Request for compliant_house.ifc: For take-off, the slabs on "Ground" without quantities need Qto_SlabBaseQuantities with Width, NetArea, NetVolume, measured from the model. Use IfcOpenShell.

First a look at what the model holds.

```python
import ifcopenshell
import ifcopenshell.util.element
import ifcopenshell.util.unit

model = ifcopenshell.open("compliant_house.ifc")
print(model.schema)
for unit_type in ("LENGTHUNIT", "AREAUNIT", "VOLUMEUNIT"):
    print(unit_type, ifcopenshell.util.unit.calculate_unit_scale(model, unit_type))
storey = next(s for s in model.by_type("IfcBuildingStorey") if s.Name == "Ground")
slabs = [e for e in ifcopenshell.util.element.get_decomposition(storey) if e.is_a("IfcSlab")]
for e in sorted(slabs, key=lambda e: e.id()):
    print(e.id(), e.is_a(), e.Name, list(ifcopenshell.util.element.get_psets(e, qtos_only=True)), sep=" | ")
```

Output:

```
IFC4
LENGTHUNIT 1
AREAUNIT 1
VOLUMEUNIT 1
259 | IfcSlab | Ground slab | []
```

```python
import ifcopenshell
import ifcopenshell.api.pset
import ifcopenshell.geom
import ifcopenshell.util.element
import ifcopenshell.util.shape
import ifcopenshell.util.unit

model = ifcopenshell.open("compliant_house.ifc")
unit_scale = ifcopenshell.util.unit.calculate_unit_scale(model)
area_scale = ifcopenshell.util.unit.calculate_unit_scale(model, "AREAUNIT")
volume_scale = ifcopenshell.util.unit.calculate_unit_scale(model, "VOLUMEUNIT")
settings = ifcopenshell.geom.settings()

storey = next(s for s in model.by_type("IfcBuildingStorey") if s.Name == "Ground")
slabs = [e for e in ifcopenshell.util.element.get_decomposition(storey) if e.is_a("IfcSlab")]

for e in sorted(slabs, key=lambda e: e.id()):
    if ifcopenshell.util.element.get_psets(e, qtos_only=True, should_inherit=False):
        continue
    # Geometry comes back in metres, in the element's own axes.
    shape = ifcopenshell.geom.create_shape(settings, e)
    values = {
        "Width": ifcopenshell.util.shape.get_z(shape.geometry) / unit_scale,
        "NetArea": ifcopenshell.util.shape.get_footprint_area(shape.geometry) / area_scale,
        "NetVolume": ifcopenshell.util.shape.get_volume(shape.geometry) / volume_scale,
    }
    qto = ifcopenshell.api.pset.add_qto(model, product=e, name="Qto_SlabBaseQuantities")
    ifcopenshell.api.pset.edit_qto(model, qto=qto, properties=values)
    print(e.id(), {k: round(v, 3) for k, v in values.items()})

model.write("compliant_house_v2.ifc")
```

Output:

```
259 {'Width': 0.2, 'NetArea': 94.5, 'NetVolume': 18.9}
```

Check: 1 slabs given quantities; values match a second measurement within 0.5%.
